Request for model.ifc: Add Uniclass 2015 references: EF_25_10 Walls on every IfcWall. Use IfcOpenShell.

First a look at what the model holds.

```python
import ifcopenshell

model = ifcopenshell.open("model.ifc")
print(model.schema)
print("classifications:", [c.Name for c in model.by_type("IfcClassification")])
for ifc_class in ("IfcDoor", "IfcRoof", "IfcStair", "IfcWall", "IfcWindow"):
    print(ifc_class, len(model.by_type(ifc_class)))
```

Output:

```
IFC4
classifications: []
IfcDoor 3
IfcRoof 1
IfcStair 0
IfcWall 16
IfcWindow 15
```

```python
import ifcopenshell
import ifcopenshell.api.classification

model = ifcopenshell.open("model.ifc")

system = ifcopenshell.api.classification.add_classification(model, classification="Uniclass 2015")

codes = {
    "IfcWall": ("EF_25_10", "Walls"),
}
for ifc_class, (code, name) in codes.items():
    products = model.by_type(ifc_class)
    ifcopenshell.api.classification.add_reference(
        model, products=products, classification=system, identification=code, name=name
    )
    print(code, len(products))

model.write("model_rev.ifc")
```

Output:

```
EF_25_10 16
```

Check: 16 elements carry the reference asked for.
